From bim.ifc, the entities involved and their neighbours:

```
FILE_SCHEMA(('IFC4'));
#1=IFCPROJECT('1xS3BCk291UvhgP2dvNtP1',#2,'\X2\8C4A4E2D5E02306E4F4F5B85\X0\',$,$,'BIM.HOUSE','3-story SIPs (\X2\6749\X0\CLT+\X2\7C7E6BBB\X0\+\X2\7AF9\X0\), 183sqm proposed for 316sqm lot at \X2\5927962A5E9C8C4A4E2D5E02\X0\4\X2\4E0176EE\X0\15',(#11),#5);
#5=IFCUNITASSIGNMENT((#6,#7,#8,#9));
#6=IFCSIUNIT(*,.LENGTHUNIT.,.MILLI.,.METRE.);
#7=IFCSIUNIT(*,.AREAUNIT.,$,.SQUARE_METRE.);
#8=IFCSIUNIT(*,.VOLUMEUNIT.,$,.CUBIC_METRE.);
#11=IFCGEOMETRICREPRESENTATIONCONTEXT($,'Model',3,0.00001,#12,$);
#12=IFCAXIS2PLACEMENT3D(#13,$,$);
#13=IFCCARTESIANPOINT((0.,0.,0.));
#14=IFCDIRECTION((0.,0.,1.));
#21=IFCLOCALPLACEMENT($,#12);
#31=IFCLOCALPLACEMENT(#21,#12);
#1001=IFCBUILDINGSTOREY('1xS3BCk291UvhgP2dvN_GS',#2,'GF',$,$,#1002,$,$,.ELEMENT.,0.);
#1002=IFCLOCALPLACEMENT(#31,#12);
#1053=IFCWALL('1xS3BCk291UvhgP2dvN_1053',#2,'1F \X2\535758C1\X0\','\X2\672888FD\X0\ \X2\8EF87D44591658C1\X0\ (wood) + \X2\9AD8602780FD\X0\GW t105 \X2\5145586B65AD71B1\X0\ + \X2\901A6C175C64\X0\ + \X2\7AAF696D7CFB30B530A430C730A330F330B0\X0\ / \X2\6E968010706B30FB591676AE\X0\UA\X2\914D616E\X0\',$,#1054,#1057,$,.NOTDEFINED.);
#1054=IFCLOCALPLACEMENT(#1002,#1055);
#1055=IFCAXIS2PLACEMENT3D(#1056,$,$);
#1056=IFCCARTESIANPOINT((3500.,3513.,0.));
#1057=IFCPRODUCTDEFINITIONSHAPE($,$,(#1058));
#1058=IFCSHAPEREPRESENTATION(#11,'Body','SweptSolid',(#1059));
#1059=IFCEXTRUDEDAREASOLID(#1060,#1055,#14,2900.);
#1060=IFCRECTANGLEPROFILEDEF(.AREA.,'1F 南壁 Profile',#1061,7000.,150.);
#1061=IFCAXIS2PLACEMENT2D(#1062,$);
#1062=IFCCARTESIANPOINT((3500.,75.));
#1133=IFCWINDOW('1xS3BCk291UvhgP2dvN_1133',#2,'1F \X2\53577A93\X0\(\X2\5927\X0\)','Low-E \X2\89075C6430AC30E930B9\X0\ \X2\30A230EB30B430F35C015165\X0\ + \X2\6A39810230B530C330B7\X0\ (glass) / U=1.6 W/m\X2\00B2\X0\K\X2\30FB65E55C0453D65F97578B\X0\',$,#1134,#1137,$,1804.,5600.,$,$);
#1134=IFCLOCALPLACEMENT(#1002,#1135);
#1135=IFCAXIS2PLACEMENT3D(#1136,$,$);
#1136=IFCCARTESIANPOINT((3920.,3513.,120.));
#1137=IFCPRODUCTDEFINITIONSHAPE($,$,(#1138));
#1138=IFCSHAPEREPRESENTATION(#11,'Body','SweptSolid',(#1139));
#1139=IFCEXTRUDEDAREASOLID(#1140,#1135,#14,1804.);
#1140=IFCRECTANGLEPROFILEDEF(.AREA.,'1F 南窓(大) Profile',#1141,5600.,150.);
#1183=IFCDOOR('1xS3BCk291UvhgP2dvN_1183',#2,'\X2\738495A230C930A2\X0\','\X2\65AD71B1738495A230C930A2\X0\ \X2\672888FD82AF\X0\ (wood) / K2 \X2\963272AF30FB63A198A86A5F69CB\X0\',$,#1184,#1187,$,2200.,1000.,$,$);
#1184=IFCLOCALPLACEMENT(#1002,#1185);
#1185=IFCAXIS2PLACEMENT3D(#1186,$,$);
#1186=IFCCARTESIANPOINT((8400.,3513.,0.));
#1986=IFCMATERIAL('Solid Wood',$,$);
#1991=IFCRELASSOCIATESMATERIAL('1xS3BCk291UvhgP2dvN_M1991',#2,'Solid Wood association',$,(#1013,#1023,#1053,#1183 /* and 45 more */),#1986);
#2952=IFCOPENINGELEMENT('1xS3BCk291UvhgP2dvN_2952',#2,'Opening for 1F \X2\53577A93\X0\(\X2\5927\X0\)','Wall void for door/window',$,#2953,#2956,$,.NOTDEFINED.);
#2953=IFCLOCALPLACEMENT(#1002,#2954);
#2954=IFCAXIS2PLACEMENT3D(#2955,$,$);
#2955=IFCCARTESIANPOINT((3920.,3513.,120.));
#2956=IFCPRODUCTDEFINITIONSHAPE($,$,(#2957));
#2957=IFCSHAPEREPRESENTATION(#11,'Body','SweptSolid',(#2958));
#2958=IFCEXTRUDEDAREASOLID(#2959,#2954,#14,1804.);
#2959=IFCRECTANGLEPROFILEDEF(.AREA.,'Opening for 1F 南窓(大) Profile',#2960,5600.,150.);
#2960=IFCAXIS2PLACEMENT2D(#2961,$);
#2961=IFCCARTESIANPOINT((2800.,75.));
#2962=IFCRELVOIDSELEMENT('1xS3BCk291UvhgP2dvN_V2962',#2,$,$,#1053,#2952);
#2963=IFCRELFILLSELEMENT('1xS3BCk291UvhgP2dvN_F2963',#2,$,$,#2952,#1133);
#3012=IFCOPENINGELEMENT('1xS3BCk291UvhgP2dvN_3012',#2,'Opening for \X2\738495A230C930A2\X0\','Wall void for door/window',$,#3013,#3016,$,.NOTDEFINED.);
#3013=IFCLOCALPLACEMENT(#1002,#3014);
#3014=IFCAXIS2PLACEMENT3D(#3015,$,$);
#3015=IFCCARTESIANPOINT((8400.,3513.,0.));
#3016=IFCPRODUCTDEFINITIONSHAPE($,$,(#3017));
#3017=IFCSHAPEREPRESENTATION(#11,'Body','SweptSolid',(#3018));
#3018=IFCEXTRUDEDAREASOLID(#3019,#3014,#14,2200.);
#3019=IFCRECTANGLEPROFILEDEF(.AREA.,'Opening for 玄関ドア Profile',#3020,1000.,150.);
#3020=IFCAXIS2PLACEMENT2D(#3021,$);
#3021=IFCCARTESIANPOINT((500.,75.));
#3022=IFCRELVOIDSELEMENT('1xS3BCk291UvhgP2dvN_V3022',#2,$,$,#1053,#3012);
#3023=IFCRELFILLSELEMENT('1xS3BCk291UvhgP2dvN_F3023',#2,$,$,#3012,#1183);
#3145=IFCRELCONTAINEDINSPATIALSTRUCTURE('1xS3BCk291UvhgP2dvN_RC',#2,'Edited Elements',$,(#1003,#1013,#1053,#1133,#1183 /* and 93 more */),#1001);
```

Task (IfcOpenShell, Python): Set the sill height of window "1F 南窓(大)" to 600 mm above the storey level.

```python
import numpy as np
import ifcopenshell
import ifcopenshell.api.geometry
import ifcopenshell.geom
import ifcopenshell.util.element
import ifcopenshell.util.placement
import ifcopenshell.util.shape
import ifcopenshell.util.unit

model = ifcopenshell.open("bim.ifc")
unit_scale = ifcopenshell.util.unit.calculate_unit_scale(model)

window = model.by_guid("1xS3BCk291UvhgP2dvN_1133")
opening = window.FillsVoids[0].RelatingOpeningElement
storey = ifcopenshell.util.element.get_container(window, ifc_class="IfcBuildingStorey")
level = ifcopenshell.util.placement.get_local_placement(storey.ObjectPlacement)[2, 3]

# The opening's origin need not be at the sill, so measure its lowest point.
shape = ifcopenshell.geom.create_shape(ifcopenshell.geom.settings(), opening)
bottom = ifcopenshell.util.shape.get_shape_bottom_elevation(shape, shape.geometry) / unit_scale
dz = level + 0.6 / unit_scale - bottom

shift = np.array([0.0, 0.0, dz])
# The window is not placed relative to its opening, so move both.
for product in (opening, window):
    matrix = ifcopenshell.util.placement.get_local_placement(product.ObjectPlacement)
    matrix[:3, 3] += shift
    ifcopenshell.api.geometry.edit_object_placement(model, product=product, matrix=matrix, is_si=False)

print(f"moved by {dz * unit_scale:+.3f} m")

model.write("bim-out.ifc")
```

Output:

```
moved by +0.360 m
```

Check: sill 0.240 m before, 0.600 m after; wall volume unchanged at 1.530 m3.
